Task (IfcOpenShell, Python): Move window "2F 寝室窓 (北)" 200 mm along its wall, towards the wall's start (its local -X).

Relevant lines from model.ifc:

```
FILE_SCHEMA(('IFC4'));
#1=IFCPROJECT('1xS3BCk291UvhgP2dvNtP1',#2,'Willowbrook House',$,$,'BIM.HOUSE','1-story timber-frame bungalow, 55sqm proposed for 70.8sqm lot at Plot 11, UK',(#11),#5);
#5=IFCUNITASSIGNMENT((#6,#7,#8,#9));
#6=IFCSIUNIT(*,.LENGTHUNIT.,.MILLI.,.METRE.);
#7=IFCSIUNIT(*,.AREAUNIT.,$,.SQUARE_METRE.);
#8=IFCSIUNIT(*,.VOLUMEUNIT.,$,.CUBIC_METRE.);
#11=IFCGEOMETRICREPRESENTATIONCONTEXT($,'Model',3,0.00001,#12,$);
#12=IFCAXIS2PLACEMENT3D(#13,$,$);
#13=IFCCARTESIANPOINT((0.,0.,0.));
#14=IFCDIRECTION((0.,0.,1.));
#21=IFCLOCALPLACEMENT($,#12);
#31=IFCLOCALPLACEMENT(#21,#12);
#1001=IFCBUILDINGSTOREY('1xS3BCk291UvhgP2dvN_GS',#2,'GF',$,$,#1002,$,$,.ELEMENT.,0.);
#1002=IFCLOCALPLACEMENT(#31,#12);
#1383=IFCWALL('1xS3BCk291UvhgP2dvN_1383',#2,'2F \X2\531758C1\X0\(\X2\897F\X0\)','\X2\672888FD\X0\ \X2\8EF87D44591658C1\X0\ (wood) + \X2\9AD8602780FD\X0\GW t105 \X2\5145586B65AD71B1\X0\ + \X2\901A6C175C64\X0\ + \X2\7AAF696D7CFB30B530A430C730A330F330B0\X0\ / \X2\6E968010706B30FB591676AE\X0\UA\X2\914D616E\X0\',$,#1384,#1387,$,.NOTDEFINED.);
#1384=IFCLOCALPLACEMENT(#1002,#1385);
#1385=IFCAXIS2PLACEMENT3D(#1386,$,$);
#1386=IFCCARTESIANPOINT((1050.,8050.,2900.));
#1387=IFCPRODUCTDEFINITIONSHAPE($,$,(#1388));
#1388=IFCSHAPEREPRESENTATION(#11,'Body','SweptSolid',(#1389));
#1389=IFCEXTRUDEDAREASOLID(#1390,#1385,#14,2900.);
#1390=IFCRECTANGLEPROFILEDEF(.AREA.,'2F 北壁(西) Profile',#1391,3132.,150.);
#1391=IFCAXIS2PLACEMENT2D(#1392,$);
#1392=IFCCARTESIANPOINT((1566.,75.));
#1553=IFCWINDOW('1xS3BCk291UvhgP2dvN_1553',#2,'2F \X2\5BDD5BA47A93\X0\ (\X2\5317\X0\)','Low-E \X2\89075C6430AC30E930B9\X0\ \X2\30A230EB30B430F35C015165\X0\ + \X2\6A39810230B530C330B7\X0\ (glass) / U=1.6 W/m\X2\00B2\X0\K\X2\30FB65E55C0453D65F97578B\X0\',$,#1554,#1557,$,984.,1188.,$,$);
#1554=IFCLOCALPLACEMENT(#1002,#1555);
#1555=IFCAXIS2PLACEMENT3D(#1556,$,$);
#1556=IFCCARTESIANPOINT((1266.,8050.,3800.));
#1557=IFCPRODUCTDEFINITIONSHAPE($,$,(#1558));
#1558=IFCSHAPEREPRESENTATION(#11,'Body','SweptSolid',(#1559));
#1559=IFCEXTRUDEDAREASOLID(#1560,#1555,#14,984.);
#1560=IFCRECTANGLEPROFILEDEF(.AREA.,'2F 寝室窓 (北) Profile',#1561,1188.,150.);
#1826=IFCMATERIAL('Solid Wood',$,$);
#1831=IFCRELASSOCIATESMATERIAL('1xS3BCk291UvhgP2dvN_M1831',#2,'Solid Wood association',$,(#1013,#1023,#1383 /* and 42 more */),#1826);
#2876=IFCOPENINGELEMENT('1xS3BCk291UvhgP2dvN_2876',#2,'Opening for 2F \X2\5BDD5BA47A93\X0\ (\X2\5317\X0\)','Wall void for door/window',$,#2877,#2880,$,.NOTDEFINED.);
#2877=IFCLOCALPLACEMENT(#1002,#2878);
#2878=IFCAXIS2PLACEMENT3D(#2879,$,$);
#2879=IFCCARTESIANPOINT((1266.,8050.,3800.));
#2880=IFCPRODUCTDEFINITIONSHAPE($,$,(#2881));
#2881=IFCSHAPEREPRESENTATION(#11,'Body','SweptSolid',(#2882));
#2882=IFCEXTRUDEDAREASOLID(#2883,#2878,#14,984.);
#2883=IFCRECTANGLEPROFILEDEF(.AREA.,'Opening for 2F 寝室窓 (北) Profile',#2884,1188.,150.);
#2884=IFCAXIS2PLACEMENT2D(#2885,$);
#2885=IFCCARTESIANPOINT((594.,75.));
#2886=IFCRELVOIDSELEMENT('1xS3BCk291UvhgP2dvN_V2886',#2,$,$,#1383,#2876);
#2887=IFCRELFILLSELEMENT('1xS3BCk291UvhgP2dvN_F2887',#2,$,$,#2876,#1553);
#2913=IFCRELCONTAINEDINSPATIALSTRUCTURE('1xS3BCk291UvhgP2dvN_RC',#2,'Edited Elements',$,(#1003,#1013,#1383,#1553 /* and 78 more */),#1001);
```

```python
import ifcopenshell
import ifcopenshell.api.geometry
import ifcopenshell.util.placement
import ifcopenshell.util.unit

model = ifcopenshell.open("model.ifc")
unit_scale = ifcopenshell.util.unit.calculate_unit_scale(model)

window = model.by_guid("1xS3BCk291UvhgP2dvN_1553")
opening = window.FillsVoids[0].RelatingOpeningElement
wall = opening.VoidsElements[0].RelatingBuildingElement

wall_matrix = ifcopenshell.util.placement.get_local_placement(wall.ObjectPlacement)
shift = wall_matrix[:3, 0] * -0.2 / unit_scale
before = ifcopenshell.util.placement.get_local_placement(window.ObjectPlacement)[:3, 3].copy()

# The window is not placed relative to its opening, so move both.
for product in (opening, window):
    matrix = ifcopenshell.util.placement.get_local_placement(product.ObjectPlacement)
    matrix[:3, 3] += shift
    ifcopenshell.api.geometry.edit_object_placement(model, product=product, matrix=matrix, is_si=False)

after = ifcopenshell.util.placement.get_local_placement(window.ObjectPlacement)[:3, 3]
print("window moved by", (after - before).round(3) + 0.0)

model.write("model_rev.ifc")
```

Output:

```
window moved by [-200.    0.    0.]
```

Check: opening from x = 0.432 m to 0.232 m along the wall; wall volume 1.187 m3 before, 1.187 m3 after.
